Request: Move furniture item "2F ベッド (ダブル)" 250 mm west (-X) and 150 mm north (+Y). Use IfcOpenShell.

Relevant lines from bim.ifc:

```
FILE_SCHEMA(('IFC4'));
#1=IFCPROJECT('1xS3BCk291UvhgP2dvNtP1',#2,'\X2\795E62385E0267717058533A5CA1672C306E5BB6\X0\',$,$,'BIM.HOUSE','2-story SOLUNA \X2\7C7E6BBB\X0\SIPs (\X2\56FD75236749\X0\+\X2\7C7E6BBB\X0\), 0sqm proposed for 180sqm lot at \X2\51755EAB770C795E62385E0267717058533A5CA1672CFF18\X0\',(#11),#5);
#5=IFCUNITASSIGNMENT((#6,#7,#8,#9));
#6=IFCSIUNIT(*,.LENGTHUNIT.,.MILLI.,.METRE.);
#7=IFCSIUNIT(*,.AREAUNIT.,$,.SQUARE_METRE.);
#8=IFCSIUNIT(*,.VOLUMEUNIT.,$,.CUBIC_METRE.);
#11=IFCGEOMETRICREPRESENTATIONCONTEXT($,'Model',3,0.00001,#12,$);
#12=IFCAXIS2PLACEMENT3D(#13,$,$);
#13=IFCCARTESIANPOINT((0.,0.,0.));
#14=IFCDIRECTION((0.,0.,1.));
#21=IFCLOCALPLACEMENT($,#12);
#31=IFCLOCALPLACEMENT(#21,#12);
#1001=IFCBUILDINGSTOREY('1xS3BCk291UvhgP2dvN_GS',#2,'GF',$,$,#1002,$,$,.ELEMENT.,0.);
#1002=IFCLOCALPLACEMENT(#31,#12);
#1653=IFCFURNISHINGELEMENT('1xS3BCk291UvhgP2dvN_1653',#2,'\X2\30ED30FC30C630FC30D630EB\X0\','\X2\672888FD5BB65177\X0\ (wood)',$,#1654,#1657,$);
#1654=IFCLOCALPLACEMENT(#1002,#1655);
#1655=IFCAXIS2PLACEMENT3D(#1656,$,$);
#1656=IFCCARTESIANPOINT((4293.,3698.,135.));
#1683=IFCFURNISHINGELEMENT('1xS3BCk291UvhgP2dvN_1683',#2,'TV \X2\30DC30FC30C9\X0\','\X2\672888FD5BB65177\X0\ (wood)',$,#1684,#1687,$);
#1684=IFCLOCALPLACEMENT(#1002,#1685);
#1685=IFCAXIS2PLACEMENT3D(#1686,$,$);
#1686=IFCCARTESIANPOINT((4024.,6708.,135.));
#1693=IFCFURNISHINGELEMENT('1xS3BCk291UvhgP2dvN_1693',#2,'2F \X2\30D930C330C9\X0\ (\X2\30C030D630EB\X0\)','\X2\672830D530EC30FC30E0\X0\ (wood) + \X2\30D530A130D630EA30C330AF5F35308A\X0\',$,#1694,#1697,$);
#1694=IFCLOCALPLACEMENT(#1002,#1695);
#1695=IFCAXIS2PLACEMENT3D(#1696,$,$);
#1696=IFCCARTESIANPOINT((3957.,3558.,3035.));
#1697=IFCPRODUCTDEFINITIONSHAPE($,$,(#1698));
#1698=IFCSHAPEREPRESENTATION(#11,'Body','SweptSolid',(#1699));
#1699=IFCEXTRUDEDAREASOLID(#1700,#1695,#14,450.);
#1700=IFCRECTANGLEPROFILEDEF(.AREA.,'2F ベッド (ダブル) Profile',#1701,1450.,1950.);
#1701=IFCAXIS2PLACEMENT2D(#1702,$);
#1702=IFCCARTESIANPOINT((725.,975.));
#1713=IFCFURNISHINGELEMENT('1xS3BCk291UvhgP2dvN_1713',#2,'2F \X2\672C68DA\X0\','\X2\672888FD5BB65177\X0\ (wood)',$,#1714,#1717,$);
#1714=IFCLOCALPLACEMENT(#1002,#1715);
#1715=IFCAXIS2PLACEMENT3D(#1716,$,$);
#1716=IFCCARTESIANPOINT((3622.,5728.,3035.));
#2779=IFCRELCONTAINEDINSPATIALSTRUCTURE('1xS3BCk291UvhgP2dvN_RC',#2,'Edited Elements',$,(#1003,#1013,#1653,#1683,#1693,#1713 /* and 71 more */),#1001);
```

```python
import ifcopenshell
import ifcopenshell.api.geometry
import ifcopenshell.util.placement

model = ifcopenshell.open("bim.ifc")

item = model.by_guid("1xS3BCk291UvhgP2dvN_1693")
matrix = ifcopenshell.util.placement.get_local_placement(item.ObjectPlacement)
matrix[0, 3] -= 250.0
matrix[1, 3] += 150.0
ifcopenshell.api.geometry.edit_object_placement(model, product=item, matrix=matrix, is_si=False)

print(ifcopenshell.util.placement.get_local_placement(item.ObjectPlacement).round(3) + 0.0)

model.write("bim_v2.ifc")
```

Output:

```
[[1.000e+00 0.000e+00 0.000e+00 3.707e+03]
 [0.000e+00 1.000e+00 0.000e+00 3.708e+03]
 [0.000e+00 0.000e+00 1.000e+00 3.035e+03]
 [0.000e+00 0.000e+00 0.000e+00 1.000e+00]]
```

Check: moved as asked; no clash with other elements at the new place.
